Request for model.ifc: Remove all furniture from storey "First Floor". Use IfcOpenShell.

First a look at what the model holds.

```python
import ifcopenshell
import ifcopenshell.util.element

model = ifcopenshell.open("model.ifc")
print(model.schema)
storey = next(s for s in model.by_type("IfcBuildingStorey") if s.Name == "First Floor")
furniture = [e for e in ifcopenshell.util.element.get_decomposition(storey) if e.is_a("IfcFurnishingElement")]
seen = {}
for e in furniture:
    element_type = ifcopenshell.util.element.get_type(e)
    name = element_type.Name if element_type not in (None, e) else None
    seen[name] = seen.get(name, 0) + 1
for name, count in sorted(seen.items(), key=str):
    print(count, "x", name)
```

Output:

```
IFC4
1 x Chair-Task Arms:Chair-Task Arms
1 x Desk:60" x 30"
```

```python
import ifcopenshell
import ifcopenshell.api.root
import ifcopenshell.util.element

model = ifcopenshell.open("model.ifc")

storey = next(s for s in model.by_type("IfcBuildingStorey") if s.Name == "First Floor")
furniture = [e for e in ifcopenshell.util.element.get_decomposition(storey) if e.is_a("IfcFurnishingElement")]

for e in furniture:
    ifcopenshell.api.root.remove_product(model, product=e)
print(len(furniture), "removed")

model.write("model-out.ifc")
```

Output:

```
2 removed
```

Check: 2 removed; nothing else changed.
